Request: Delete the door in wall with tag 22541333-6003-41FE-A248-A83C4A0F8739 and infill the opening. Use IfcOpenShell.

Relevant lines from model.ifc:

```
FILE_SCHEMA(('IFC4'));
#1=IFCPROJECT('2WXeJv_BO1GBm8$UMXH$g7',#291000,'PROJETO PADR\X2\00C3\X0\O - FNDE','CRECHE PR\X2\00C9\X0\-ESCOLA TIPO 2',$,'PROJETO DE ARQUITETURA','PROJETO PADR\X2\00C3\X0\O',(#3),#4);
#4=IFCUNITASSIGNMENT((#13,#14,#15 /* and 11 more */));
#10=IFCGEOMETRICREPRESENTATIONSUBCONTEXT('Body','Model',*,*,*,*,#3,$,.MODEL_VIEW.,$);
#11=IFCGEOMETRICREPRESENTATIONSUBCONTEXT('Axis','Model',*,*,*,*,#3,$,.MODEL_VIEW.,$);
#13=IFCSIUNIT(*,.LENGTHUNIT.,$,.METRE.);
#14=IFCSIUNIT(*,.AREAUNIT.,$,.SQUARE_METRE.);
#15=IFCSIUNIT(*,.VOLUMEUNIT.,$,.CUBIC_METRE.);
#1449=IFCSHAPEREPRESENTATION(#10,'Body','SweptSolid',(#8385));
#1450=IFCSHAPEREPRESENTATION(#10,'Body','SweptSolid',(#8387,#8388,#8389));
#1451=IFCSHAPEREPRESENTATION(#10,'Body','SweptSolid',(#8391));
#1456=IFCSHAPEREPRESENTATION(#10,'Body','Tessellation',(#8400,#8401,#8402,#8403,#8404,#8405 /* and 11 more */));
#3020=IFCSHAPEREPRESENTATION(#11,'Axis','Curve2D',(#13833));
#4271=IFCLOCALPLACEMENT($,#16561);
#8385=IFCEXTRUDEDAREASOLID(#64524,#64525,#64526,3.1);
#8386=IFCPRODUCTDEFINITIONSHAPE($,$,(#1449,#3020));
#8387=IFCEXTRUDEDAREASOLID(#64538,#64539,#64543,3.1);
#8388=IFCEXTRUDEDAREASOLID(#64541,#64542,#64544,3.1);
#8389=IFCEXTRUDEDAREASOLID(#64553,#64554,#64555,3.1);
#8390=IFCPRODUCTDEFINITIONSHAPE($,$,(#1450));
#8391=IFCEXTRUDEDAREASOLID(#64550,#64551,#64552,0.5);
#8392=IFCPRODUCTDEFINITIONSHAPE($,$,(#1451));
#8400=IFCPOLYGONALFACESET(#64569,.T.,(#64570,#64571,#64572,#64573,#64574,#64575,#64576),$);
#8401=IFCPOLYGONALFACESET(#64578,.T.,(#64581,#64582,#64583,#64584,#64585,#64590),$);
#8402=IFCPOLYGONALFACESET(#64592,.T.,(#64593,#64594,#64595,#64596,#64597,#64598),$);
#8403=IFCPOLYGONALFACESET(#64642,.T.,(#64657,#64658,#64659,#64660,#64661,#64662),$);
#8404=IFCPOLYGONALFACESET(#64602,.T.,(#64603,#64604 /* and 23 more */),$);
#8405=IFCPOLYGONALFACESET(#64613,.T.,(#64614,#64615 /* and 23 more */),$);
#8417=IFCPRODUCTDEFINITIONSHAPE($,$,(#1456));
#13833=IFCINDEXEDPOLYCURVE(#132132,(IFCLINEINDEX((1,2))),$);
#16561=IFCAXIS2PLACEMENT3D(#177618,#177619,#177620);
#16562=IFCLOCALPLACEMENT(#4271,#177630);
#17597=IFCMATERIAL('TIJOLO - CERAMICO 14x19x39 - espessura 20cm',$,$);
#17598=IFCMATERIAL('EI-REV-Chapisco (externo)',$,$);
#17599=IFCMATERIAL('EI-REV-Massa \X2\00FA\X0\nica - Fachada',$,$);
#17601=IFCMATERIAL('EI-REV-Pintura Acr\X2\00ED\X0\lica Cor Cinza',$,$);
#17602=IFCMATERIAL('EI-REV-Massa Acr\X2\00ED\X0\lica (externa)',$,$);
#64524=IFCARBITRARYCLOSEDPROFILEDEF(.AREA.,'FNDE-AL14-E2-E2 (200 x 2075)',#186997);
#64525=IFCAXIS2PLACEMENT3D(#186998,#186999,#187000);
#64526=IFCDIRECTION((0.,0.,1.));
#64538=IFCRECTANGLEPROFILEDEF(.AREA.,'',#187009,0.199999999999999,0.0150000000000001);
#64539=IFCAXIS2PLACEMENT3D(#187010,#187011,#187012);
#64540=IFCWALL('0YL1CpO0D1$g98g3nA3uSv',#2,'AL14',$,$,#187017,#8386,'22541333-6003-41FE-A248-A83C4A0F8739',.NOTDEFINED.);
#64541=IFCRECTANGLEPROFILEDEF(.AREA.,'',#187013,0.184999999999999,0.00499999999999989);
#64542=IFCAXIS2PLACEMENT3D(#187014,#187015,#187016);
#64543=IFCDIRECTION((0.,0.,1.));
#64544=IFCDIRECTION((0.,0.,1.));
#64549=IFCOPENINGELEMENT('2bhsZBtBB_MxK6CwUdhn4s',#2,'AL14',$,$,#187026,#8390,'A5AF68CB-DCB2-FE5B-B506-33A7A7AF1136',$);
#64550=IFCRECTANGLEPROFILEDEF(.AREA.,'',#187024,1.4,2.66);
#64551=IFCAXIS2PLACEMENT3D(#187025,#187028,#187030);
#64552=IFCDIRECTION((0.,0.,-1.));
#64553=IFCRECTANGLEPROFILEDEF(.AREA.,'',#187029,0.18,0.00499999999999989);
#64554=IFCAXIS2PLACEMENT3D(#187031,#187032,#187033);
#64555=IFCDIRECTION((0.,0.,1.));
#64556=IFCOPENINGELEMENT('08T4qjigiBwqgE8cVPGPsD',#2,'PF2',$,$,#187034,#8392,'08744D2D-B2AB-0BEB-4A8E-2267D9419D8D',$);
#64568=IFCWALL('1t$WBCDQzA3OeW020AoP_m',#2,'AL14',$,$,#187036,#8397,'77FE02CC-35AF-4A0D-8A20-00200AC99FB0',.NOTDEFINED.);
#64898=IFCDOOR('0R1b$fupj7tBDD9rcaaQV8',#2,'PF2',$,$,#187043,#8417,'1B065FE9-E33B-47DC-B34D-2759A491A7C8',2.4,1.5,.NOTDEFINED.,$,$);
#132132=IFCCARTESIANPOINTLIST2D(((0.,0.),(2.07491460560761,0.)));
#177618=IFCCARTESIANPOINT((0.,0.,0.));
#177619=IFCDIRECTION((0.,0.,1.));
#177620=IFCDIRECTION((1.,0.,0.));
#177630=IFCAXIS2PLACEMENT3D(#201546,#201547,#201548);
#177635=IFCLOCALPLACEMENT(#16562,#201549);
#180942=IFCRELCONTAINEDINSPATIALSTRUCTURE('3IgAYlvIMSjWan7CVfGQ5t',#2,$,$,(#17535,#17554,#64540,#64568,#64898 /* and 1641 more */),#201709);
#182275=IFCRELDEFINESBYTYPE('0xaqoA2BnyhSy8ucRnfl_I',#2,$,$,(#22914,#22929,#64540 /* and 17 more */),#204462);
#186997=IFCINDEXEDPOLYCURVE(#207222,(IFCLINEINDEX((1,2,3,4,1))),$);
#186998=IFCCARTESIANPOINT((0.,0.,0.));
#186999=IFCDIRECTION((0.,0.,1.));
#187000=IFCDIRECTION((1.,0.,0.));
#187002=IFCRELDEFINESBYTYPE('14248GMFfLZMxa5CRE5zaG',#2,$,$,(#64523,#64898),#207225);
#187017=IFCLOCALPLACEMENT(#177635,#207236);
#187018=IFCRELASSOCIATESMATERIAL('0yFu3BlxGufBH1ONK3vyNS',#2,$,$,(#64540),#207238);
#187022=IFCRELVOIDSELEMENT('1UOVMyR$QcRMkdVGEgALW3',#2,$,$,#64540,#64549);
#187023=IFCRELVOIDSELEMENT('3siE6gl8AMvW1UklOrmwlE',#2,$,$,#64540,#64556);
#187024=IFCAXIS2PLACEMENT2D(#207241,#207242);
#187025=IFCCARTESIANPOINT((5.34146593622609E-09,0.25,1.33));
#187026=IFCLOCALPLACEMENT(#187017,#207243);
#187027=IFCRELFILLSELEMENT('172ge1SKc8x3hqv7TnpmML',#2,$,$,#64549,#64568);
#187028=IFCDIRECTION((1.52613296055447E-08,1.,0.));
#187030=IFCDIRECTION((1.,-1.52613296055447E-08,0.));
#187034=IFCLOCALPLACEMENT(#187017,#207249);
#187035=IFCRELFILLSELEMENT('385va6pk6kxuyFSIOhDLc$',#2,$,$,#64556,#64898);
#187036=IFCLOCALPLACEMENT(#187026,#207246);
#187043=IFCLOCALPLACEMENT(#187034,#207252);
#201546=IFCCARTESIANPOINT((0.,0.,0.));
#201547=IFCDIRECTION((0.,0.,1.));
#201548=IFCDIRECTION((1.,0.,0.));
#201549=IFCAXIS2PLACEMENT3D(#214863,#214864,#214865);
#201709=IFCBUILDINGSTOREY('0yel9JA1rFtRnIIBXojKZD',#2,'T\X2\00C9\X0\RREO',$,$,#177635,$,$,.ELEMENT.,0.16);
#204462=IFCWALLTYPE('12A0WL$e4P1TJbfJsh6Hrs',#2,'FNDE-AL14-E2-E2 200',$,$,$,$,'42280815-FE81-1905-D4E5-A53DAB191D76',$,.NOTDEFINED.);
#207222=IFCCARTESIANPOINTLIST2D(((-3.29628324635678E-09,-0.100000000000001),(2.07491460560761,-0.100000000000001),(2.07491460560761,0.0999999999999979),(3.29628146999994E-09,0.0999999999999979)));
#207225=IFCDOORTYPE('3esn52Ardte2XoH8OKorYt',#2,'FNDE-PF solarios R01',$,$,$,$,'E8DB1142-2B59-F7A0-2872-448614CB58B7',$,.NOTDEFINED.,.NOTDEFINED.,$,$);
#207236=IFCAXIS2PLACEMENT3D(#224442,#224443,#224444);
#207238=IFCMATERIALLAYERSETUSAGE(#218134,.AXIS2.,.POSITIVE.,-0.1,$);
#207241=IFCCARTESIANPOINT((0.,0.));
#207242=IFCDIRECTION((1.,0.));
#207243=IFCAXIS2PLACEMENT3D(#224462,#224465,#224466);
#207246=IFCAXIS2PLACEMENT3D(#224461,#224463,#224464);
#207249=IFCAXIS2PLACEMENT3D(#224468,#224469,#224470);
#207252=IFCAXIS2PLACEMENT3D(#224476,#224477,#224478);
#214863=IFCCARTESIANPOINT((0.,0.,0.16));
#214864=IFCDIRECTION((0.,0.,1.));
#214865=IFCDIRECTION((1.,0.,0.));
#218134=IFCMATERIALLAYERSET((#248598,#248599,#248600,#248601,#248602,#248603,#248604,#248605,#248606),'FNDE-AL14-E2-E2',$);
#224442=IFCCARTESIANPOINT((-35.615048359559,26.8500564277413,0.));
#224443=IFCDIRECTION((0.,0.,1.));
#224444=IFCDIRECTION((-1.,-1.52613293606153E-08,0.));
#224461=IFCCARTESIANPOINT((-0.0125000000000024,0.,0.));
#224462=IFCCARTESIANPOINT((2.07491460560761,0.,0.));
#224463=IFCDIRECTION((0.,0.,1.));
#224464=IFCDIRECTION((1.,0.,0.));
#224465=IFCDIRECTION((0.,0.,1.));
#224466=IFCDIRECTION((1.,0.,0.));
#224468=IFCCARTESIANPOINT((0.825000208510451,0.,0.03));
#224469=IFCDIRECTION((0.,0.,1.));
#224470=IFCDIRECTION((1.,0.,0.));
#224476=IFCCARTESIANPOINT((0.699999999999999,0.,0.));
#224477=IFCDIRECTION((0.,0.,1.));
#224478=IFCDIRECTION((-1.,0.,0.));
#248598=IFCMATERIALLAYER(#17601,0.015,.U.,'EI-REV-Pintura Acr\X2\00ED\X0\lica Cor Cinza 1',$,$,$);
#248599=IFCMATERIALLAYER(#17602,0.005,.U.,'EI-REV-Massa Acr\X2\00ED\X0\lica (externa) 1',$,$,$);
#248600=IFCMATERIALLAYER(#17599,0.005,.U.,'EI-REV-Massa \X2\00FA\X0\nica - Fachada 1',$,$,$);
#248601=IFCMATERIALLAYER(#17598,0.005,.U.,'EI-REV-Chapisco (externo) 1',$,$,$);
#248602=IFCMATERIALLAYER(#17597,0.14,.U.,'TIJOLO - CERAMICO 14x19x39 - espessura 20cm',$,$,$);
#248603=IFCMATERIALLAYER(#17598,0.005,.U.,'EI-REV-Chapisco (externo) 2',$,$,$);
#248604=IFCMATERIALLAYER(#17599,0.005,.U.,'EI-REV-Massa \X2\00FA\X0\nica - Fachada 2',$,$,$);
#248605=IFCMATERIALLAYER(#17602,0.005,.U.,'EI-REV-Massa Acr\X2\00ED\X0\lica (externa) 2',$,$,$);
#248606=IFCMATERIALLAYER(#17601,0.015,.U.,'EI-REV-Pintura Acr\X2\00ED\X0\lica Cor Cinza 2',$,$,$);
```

```python
import ifcopenshell
import ifcopenshell.api.feature
import ifcopenshell.api.root
import ifcopenshell.geom
import ifcopenshell.util.shape

model = ifcopenshell.open("model.ifc")
settings = ifcopenshell.geom.settings()


def volume(element):
    """Net volume in cubic metres, openings subtracted."""
    shape = ifcopenshell.geom.create_shape(settings, element)
    return ifcopenshell.util.shape.get_volume(shape.geometry)


door = model.by_id(64898)
opening = door.FillsVoids[0].RelatingOpeningElement
wall = opening.VoidsElements[0].RelatingBuildingElement
before = volume(wall)

ifcopenshell.api.root.remove_product(model, product=door)
ifcopenshell.api.feature.remove_feature(model, feature=opening)

after = volume(wall)

print(f"wall volume {before:.3f} -> {after:.3f} m3")

model.write("model_updated.ifc")
```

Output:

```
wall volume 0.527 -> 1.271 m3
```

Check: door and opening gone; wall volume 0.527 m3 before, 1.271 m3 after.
